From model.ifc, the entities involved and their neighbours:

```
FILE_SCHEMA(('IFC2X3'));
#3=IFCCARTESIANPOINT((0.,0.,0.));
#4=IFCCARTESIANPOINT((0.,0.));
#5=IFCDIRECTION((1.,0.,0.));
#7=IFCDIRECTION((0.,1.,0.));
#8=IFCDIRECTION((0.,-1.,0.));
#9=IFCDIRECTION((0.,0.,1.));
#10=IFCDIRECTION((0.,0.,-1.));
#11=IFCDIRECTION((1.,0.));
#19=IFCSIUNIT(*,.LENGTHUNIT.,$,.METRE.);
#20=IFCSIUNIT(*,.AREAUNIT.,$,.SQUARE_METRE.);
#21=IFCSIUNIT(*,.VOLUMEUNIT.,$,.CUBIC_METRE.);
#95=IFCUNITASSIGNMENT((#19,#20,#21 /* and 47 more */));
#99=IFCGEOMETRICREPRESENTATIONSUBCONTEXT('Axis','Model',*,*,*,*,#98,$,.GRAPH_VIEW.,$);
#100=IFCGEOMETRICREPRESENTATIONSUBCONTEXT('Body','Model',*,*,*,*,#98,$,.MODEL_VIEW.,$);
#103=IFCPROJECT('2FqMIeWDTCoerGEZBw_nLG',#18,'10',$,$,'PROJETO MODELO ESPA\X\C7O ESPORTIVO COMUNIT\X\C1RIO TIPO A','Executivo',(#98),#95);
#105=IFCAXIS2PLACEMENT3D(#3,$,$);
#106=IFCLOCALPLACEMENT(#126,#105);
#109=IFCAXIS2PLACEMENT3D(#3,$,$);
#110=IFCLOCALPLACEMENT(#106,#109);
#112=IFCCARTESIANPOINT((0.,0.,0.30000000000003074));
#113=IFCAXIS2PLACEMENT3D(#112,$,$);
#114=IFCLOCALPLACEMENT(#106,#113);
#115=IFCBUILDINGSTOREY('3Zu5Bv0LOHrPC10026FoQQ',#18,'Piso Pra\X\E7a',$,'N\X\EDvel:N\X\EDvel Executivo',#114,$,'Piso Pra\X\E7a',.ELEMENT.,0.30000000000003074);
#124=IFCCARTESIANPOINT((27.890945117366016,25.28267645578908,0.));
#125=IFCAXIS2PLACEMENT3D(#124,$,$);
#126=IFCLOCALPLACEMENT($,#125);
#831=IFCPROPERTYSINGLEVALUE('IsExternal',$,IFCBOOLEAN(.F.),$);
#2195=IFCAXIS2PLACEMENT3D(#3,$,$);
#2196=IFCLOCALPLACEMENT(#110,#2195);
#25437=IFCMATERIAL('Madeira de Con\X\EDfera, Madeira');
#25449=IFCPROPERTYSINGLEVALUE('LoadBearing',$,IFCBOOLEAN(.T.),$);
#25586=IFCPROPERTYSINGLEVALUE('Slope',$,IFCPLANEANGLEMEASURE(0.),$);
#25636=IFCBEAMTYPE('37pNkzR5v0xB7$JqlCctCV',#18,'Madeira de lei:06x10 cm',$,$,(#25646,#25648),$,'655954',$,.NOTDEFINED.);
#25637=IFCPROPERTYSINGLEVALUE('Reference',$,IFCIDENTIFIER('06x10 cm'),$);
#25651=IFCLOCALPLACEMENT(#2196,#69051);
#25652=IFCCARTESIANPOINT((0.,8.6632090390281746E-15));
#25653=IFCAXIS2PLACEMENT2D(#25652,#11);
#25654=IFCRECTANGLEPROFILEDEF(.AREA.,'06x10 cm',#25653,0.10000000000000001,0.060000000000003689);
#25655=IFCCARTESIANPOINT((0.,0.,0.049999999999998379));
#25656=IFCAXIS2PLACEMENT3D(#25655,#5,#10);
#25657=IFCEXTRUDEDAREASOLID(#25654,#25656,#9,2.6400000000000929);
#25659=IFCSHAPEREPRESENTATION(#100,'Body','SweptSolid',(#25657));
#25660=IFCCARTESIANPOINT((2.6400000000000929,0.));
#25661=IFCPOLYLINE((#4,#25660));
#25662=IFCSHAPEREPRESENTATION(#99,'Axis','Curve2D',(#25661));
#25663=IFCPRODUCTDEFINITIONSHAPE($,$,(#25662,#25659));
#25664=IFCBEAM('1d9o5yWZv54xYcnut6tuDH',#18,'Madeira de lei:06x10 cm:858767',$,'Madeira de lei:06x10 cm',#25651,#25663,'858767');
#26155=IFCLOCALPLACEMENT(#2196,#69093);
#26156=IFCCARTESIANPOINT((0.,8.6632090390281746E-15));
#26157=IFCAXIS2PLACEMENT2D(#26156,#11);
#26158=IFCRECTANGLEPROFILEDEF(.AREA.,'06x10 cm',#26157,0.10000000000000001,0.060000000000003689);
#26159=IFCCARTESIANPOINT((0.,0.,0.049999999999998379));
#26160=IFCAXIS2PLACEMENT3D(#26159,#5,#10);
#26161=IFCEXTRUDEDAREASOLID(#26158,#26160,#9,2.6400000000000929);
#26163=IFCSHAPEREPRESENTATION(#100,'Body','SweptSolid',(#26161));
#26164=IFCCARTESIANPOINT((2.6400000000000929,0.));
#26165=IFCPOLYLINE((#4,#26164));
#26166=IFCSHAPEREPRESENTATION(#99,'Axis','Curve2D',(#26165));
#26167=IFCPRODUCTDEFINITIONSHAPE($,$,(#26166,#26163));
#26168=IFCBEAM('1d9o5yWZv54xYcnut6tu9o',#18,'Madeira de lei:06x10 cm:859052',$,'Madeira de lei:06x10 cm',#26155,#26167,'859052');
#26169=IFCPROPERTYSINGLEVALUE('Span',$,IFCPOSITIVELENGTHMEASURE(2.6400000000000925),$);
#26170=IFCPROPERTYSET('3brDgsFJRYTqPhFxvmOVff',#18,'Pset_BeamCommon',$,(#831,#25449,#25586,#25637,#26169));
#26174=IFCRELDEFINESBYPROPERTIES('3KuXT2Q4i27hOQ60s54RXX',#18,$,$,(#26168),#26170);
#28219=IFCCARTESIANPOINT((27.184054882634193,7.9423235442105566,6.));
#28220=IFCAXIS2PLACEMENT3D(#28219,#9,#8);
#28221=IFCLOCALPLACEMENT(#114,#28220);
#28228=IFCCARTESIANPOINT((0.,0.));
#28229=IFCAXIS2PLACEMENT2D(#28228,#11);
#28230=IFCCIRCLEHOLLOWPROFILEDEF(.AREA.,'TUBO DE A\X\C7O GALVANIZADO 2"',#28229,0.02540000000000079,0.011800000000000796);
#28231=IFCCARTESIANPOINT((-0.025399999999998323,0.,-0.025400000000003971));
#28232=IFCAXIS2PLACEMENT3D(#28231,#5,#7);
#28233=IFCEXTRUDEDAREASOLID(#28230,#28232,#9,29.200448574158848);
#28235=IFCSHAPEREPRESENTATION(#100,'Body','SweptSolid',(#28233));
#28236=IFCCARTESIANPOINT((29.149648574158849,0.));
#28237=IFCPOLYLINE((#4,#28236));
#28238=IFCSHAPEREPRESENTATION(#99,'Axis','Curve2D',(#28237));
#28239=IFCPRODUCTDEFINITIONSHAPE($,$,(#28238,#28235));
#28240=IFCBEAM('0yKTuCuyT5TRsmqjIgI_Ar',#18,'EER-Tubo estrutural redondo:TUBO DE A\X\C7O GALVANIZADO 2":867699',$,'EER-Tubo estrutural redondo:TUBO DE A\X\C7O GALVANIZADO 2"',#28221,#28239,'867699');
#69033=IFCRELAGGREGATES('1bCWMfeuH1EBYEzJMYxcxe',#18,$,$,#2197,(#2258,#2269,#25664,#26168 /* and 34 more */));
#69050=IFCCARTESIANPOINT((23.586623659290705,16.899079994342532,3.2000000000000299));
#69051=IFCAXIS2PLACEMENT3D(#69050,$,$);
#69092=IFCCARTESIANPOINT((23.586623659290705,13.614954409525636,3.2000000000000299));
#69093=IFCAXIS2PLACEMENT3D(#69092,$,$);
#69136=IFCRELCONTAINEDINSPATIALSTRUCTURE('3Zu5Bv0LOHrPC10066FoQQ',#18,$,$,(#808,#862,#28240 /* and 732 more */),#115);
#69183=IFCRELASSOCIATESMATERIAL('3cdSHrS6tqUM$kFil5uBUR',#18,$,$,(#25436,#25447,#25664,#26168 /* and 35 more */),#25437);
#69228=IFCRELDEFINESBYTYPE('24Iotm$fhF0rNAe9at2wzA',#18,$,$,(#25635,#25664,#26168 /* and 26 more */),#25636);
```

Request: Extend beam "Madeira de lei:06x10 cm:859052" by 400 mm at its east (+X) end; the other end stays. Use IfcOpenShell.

```python
import numpy as np
import ifcopenshell
import ifcopenshell.api.pset
import ifcopenshell.util.element
import ifcopenshell.util.representation
import ifcopenshell.util.unit

model = ifcopenshell.open("model.ifc")
unit_scale = ifcopenshell.util.unit.calculate_unit_scale(model)

member = model.by_id(26168)
change = 0.4 / unit_scale

# The extrusion runs towards the end named, so only its depth changes.
body = ifcopenshell.util.representation.get_representation(member, "Model", "Body")
solid = body.Items[0]
old_length = solid.Depth
solid.Depth += change

# Move the axis end point with it.
axis = next(r for r in member.Representation.Representations if r.RepresentationIdentifier == "Axis").Items[0]
start, end = (np.array(p.Coordinates) for p in axis.Points)
end = end + (end - start) / np.linalg.norm(end - start) * change
point = model.createIfcCartesianPoint(end.tolist())
axis.Points = [axis.Points[0], point]

# Update the stored length and volume.
pset = model.by_id(ifcopenshell.util.element.get_pset(member, "Pset_BeamCommon", should_inherit=False)["id"])
ifcopenshell.api.pset.edit_pset(model, pset=pset, properties={
    "Span": model.create_entity("IfcPositiveLengthMeasure", solid.Depth),
})

print(f"length {old_length:g} -> {solid.Depth:g}")

model.write("model_updated.ifc")
```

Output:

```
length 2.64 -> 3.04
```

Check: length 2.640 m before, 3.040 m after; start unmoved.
